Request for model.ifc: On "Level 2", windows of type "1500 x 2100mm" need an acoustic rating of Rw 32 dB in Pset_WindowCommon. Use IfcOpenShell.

First a look at what the model holds.

```python
import ifcopenshell
import ifcopenshell.util.element

model = ifcopenshell.open("model.ifc")
print(model.schema)
storey = next(s for s in model.by_type("IfcBuildingStorey") if s.Name == "Level 2")
windows = [e for e in ifcopenshell.util.element.get_decomposition(storey) if e.is_a("IfcWindow")]
seen = {}
for e in windows:
    element_type = ifcopenshell.util.element.get_type(e)
    key = (element_type.Name if element_type != e and element_type else None, ifcopenshell.util.element.get_pset(e, "Pset_WindowCommon", "AcousticRating"))
    seen[key] = seen.get(key, 0) + 1
for (name, value), count in sorted(seen.items(), key=str):
    print(count, "x", name, "|", value)
```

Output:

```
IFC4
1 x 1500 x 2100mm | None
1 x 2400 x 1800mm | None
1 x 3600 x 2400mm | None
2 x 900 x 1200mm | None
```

```python
import ifcopenshell
import ifcopenshell.api.pset
import ifcopenshell.util.element

model = ifcopenshell.open("model.ifc")

storey = next(s for s in model.by_type("IfcBuildingStorey") if s.Name == "Level 2")
windows = [e for e in ifcopenshell.util.element.get_decomposition(storey) if e.is_a("IfcWindow")]

count = 0
for e in windows:
    element_type = ifcopenshell.util.element.get_type(e)
    if element_type in (None, e) or element_type.Name != "1500 x 2100mm":
        continue
    # add_pset returns the element's existing set when there is one.
    pset = ifcopenshell.api.pset.add_pset(model, product=e, name="Pset_WindowCommon")
    ifcopenshell.api.pset.edit_pset(model, pset=pset, properties={"AcousticRating": "Rw 32 dB"})
    count += 1

print(count, "windows updated")

model.write("model_edited.ifc")
```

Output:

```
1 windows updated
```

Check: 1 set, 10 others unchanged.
